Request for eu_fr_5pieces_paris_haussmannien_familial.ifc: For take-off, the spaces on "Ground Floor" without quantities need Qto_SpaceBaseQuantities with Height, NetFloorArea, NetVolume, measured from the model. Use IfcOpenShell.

First a look at what the model holds.

```python
import ifcopenshell
import ifcopenshell.util.element
import ifcopenshell.util.unit

model = ifcopenshell.open("eu_fr_5pieces_paris_haussmannien_familial.ifc")
print(model.schema)
for unit_type in ("LENGTHUNIT", "AREAUNIT", "VOLUMEUNIT"):
    print(unit_type, ifcopenshell.util.unit.calculate_unit_scale(model, unit_type))
storey = next(s for s in model.by_type("IfcBuildingStorey") if s.Name == "Ground Floor")
spaces = [e for e in ifcopenshell.util.element.get_decomposition(storey) if e.is_a("IfcSpace")]
for e in sorted(spaces, key=lambda e: e.id()):
    print(e.id(), e.is_a(), e.Name, list(ifcopenshell.util.element.get_psets(e, qtos_only=True)), sep=" | ")
```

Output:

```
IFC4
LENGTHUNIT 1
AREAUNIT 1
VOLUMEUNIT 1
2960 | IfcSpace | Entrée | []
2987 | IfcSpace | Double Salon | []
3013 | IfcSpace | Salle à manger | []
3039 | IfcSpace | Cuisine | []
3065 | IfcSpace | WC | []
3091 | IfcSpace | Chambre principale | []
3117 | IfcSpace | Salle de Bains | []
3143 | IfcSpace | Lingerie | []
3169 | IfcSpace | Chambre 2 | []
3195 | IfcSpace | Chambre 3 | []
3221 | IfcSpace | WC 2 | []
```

```python
import ifcopenshell
import ifcopenshell.api.pset
import ifcopenshell.geom
import ifcopenshell.util.element
import ifcopenshell.util.shape
import ifcopenshell.util.unit

model = ifcopenshell.open("eu_fr_5pieces_paris_haussmannien_familial.ifc")
unit_scale = ifcopenshell.util.unit.calculate_unit_scale(model)
area_scale = ifcopenshell.util.unit.calculate_unit_scale(model, "AREAUNIT")
volume_scale = ifcopenshell.util.unit.calculate_unit_scale(model, "VOLUMEUNIT")
settings = ifcopenshell.geom.settings()

storey = next(s for s in model.by_type("IfcBuildingStorey") if s.Name == "Ground Floor")
spaces = [e for e in ifcopenshell.util.element.get_decomposition(storey) if e.is_a("IfcSpace")]

for e in sorted(spaces, key=lambda e: e.id()):
    if ifcopenshell.util.element.get_psets(e, qtos_only=True, should_inherit=False):
        continue
    # Geometry comes back in metres, in the element's own axes.
    shape = ifcopenshell.geom.create_shape(settings, e)
    values = {
        "Height": ifcopenshell.util.shape.get_z(shape.geometry) / unit_scale,
        "NetFloorArea": ifcopenshell.util.shape.get_footprint_area(shape.geometry) / area_scale,
        "NetVolume": ifcopenshell.util.shape.get_volume(shape.geometry) / volume_scale,
    }
    qto = ifcopenshell.api.pset.add_qto(model, product=e, name="Qto_SpaceBaseQuantities")
    ifcopenshell.api.pset.edit_qto(model, qto=qto, properties=values)
    print(e.id(), {k: round(v, 3) for k, v in values.items()})

model.write("eu_fr_5pieces_paris_haussmannien_familial_rev.ifc")
```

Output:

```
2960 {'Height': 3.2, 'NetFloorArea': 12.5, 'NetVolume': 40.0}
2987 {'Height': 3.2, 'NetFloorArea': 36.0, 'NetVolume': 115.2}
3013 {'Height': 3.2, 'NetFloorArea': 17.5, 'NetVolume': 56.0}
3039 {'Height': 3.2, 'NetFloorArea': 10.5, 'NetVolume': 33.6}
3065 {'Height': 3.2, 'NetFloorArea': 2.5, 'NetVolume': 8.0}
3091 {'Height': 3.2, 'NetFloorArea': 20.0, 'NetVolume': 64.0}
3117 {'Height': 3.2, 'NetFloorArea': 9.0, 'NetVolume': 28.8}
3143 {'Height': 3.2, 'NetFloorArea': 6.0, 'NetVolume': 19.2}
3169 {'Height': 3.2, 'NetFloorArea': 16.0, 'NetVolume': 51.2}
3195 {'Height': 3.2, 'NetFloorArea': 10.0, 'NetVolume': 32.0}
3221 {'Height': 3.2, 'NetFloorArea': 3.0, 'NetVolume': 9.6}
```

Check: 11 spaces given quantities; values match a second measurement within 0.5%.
